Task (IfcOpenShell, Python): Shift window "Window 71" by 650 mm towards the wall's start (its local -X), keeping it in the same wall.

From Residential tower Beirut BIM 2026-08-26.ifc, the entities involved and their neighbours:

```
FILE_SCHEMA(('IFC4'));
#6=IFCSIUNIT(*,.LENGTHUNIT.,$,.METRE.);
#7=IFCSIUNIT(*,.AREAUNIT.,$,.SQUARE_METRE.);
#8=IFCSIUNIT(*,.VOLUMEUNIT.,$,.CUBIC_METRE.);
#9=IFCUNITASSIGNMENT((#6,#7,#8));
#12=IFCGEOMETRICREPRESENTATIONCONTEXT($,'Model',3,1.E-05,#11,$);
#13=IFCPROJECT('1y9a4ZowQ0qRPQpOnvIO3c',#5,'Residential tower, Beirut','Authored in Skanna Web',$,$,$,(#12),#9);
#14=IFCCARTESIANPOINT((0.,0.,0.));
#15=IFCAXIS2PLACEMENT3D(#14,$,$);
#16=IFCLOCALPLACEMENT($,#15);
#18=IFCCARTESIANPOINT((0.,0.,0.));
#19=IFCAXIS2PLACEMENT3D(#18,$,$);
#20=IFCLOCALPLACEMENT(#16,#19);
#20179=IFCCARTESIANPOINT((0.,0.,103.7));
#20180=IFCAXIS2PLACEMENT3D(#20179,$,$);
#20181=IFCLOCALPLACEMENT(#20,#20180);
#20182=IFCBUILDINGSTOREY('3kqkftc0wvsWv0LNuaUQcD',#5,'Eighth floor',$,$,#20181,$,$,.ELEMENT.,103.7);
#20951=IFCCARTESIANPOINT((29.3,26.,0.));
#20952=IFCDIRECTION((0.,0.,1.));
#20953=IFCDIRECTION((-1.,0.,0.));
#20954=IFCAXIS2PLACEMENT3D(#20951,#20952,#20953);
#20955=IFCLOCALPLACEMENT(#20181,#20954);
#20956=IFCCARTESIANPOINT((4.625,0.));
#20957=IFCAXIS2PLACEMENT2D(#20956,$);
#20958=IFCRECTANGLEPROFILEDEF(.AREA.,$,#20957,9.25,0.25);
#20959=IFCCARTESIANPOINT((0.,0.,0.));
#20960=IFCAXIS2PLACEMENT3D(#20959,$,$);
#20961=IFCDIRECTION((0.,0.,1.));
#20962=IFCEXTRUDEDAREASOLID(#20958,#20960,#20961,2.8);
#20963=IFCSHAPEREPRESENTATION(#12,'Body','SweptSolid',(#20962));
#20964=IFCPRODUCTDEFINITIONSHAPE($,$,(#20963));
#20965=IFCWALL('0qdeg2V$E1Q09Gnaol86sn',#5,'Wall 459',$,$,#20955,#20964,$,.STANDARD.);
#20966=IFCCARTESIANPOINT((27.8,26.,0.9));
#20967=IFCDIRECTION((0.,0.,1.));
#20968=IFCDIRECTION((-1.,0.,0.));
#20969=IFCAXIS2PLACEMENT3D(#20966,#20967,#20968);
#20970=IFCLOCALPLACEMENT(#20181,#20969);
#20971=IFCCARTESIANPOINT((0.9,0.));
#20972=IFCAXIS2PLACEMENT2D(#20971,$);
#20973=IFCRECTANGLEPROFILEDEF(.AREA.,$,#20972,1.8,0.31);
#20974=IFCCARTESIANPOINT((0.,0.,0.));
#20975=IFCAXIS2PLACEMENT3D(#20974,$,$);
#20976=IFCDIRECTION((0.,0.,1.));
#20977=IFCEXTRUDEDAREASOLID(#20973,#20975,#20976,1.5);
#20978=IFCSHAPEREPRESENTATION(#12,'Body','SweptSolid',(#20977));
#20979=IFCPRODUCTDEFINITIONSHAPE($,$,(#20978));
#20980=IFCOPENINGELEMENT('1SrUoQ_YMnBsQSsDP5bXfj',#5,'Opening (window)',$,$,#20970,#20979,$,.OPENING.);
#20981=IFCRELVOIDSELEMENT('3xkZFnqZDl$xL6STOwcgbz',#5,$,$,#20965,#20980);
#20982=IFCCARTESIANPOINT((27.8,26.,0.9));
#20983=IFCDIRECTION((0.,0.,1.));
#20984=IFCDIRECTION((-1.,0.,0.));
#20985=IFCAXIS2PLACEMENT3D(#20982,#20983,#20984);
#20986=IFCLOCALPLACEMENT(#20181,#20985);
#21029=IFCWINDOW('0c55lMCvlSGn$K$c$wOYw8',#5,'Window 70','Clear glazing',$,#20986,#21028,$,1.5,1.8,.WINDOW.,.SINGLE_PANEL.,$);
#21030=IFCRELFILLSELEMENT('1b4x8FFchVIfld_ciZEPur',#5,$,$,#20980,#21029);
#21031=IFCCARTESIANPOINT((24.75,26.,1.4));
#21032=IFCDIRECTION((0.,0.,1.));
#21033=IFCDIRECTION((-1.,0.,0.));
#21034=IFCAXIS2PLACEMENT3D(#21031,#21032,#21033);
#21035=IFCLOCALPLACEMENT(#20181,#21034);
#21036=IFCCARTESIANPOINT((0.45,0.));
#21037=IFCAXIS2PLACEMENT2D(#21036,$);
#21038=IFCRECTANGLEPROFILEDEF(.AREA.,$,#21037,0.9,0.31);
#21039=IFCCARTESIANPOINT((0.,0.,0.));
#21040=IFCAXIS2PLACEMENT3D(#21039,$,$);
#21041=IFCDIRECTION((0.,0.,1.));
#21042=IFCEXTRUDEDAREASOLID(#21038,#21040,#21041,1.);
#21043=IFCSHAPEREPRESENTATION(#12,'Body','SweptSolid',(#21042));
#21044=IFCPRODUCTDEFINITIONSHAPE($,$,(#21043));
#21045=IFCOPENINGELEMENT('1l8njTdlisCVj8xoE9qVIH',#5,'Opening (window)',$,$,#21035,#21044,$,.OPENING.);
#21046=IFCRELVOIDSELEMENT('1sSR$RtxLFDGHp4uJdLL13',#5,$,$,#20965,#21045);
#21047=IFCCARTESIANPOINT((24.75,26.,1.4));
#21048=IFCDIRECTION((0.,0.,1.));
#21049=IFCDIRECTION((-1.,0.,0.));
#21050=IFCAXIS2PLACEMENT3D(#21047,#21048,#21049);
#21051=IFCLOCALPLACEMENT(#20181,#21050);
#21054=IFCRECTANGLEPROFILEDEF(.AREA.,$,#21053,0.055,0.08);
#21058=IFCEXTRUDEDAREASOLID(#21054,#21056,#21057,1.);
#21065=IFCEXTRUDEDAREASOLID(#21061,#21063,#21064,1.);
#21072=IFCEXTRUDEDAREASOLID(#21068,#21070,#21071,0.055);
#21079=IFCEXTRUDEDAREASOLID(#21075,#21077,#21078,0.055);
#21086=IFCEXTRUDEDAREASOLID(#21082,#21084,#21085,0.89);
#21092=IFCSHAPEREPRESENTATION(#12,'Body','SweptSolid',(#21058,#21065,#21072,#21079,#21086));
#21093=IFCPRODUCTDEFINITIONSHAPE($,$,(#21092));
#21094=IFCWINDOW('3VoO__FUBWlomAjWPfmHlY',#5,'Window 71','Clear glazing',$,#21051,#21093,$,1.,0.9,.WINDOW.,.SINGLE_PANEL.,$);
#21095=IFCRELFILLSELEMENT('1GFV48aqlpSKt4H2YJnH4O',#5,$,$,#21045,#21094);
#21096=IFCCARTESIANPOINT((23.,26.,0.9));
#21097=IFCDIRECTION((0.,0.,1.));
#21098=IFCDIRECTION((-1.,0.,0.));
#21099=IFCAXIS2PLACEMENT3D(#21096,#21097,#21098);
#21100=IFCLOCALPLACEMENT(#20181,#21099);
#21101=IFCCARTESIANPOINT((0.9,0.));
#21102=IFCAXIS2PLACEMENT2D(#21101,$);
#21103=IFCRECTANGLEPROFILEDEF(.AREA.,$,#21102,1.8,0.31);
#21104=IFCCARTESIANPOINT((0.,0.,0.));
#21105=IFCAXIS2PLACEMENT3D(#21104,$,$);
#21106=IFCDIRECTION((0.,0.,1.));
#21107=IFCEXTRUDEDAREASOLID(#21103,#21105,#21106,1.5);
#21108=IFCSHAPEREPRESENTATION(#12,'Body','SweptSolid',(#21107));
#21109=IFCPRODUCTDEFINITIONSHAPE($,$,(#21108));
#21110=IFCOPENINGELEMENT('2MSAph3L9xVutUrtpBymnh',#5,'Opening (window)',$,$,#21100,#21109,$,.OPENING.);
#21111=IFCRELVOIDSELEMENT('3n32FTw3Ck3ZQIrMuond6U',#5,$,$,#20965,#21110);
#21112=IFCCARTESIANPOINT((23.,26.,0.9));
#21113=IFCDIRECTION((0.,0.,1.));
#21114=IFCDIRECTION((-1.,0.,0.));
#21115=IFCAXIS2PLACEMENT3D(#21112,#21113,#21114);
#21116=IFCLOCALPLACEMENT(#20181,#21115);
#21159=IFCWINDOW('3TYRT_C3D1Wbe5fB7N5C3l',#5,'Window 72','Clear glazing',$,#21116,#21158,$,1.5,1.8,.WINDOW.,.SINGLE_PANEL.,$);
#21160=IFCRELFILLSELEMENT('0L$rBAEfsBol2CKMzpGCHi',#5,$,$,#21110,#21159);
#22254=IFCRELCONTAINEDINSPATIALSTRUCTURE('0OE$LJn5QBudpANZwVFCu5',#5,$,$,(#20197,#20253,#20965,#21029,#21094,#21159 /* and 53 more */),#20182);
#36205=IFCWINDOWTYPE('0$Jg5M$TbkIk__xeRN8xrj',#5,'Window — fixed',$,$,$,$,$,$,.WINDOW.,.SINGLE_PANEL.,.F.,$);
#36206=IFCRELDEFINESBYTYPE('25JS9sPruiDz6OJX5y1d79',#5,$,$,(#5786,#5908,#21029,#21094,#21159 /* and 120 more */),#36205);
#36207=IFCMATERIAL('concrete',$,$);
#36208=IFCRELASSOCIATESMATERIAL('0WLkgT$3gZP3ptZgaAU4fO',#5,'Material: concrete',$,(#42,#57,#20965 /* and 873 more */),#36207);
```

```python
import ifcopenshell
import ifcopenshell.api.geometry
import ifcopenshell.util.placement

model = ifcopenshell.open("Residential tower Beirut BIM 2026-08-26.ifc")

window = model.by_guid("3VoO__FUBWlomAjWPfmHlY")
opening = window.FillsVoids[0].RelatingOpeningElement
wall = opening.VoidsElements[0].RelatingBuildingElement

wall_matrix = ifcopenshell.util.placement.get_local_placement(wall.ObjectPlacement)
shift = wall_matrix[:3, 0] * -0.65
before = ifcopenshell.util.placement.get_local_placement(window.ObjectPlacement)[:3, 3].copy()

# The window is not placed relative to its opening, so move both.
for product in (opening, window):
    matrix = ifcopenshell.util.placement.get_local_placement(product.ObjectPlacement)
    matrix[:3, 3] += shift
    ifcopenshell.api.geometry.edit_object_placement(model, product=product, matrix=matrix, is_si=False)

after = ifcopenshell.util.placement.get_local_placement(window.ObjectPlacement)[:3, 3]
print("window moved by", (after - before).round(3) + 0.0)

model.write("Residential tower Beirut BIM 2026-08-26_rev.ifc")
```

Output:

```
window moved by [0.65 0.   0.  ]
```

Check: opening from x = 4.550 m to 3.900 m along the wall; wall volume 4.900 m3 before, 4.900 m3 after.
